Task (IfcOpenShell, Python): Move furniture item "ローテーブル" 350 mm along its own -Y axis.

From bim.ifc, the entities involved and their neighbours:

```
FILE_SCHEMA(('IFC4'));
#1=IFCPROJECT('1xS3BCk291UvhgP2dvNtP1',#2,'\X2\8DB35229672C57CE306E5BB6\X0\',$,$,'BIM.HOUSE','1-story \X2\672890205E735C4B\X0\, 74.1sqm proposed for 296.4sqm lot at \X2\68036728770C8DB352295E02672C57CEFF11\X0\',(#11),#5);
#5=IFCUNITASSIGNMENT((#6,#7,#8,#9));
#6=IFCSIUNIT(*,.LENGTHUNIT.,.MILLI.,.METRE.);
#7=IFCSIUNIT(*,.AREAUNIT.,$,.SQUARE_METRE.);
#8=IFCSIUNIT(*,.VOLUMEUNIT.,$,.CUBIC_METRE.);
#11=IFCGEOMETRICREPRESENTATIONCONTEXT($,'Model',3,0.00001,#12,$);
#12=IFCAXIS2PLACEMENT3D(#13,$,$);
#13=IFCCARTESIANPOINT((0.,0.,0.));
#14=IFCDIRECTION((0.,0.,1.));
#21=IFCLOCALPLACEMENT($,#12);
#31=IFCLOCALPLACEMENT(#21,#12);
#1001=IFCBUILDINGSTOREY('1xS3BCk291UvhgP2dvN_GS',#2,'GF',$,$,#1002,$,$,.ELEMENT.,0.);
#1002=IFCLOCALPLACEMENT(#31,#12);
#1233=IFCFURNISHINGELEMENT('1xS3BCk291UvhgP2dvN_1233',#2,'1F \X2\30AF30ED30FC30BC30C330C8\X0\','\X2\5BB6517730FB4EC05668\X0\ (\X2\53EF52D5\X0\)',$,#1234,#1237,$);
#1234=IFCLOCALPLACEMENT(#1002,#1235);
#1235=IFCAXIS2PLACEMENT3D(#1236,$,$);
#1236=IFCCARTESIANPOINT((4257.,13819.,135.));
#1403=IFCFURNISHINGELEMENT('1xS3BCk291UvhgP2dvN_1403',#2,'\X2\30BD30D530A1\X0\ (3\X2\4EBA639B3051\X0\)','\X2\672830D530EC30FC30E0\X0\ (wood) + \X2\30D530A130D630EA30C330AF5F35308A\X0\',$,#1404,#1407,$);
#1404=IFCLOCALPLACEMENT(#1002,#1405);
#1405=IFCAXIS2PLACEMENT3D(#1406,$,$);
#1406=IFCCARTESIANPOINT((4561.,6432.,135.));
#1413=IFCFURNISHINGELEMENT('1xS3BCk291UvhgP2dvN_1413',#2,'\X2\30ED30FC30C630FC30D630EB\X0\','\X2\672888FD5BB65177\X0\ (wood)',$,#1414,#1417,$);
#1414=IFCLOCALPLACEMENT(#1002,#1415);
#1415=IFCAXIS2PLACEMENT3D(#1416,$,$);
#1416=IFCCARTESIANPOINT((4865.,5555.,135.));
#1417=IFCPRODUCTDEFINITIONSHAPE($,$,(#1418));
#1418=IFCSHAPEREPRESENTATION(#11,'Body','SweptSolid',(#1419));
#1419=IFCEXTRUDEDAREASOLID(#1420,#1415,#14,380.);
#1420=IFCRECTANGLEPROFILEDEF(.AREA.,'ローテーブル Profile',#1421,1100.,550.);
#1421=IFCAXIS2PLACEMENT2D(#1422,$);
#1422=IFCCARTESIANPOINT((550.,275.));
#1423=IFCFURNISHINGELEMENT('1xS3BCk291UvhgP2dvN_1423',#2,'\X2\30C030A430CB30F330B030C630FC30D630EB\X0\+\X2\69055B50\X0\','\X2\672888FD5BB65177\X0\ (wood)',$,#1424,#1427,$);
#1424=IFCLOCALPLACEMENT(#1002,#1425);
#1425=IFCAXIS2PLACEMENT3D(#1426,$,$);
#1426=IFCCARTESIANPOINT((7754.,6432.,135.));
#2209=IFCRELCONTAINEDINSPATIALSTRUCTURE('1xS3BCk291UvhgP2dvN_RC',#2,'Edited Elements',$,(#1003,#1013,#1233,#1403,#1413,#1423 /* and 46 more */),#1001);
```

```python
import ifcopenshell
import ifcopenshell.api.geometry
import ifcopenshell.util.placement
import ifcopenshell.util.unit

model = ifcopenshell.open("bim.ifc")
unit_scale = ifcopenshell.util.unit.calculate_unit_scale(model)

item = model.by_guid("1xS3BCk291UvhgP2dvN_1413")
matrix = ifcopenshell.util.placement.get_local_placement(item.ObjectPlacement)
matrix[:3, 3] -= matrix[:3, 1] * 0.35 / unit_scale
ifcopenshell.api.geometry.edit_object_placement(model, product=item, matrix=matrix, is_si=False)

print(ifcopenshell.util.placement.get_local_placement(item.ObjectPlacement).round(3) + 0.0)

model.write("bim_rev.ifc")
```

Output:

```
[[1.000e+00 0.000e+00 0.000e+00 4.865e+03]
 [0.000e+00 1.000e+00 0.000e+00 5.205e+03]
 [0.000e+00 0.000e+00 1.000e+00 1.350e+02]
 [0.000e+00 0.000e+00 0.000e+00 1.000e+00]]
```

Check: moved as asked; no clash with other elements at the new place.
